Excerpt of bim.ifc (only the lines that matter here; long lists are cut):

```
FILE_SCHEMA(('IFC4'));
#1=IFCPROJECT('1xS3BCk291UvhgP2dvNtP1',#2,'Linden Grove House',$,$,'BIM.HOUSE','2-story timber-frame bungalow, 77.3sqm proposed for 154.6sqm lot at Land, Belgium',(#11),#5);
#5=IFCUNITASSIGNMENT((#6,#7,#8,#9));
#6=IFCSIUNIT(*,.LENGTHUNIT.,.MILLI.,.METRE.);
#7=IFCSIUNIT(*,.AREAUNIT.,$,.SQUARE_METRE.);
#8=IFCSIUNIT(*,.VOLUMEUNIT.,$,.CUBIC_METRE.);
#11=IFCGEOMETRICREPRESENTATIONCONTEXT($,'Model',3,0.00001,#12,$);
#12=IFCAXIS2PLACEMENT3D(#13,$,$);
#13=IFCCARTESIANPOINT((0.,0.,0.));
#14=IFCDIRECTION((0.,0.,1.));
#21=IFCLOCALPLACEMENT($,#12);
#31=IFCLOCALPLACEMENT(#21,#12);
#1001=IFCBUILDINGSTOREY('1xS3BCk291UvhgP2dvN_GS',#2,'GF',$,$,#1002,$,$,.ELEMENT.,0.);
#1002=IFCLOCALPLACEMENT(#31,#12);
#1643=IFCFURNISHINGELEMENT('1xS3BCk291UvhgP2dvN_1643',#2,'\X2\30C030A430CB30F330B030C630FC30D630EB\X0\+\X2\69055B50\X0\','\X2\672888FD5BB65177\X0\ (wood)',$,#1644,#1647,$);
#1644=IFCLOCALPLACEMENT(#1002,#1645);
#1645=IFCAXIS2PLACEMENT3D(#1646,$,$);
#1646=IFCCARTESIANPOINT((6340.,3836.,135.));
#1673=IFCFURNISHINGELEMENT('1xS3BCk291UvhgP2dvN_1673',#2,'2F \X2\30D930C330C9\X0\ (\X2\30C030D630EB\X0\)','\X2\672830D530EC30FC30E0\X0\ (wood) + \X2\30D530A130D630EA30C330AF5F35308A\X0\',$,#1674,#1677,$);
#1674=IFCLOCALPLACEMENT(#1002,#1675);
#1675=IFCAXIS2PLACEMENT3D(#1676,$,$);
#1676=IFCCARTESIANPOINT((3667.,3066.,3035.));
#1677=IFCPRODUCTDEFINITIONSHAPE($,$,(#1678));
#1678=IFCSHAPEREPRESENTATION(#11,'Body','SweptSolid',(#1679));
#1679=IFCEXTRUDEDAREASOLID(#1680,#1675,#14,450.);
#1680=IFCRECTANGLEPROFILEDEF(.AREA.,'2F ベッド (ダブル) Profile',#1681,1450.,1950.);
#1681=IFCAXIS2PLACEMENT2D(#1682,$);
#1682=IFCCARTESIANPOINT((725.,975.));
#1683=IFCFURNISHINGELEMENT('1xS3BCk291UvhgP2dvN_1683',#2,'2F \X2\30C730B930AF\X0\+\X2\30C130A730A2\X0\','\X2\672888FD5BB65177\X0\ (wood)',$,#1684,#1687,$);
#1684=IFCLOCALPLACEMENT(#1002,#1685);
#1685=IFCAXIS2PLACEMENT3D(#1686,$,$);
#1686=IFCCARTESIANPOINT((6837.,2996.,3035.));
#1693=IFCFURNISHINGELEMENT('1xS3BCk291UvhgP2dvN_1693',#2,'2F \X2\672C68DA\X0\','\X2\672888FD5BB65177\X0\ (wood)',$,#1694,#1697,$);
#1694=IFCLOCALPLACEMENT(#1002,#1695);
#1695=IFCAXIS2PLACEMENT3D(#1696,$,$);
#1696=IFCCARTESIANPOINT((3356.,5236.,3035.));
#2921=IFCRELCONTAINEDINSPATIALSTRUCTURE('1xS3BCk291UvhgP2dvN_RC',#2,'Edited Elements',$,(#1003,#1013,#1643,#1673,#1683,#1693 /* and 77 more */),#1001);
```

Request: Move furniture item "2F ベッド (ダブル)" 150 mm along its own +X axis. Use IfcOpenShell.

```python
import ifcopenshell
import ifcopenshell.api.geometry
import ifcopenshell.util.placement
import ifcopenshell.util.unit

model = ifcopenshell.open("bim.ifc")
unit_scale = ifcopenshell.util.unit.calculate_unit_scale(model)

item = model.by_id(1673)
matrix = ifcopenshell.util.placement.get_local_placement(item.ObjectPlacement)
matrix[:3, 3] += matrix[:3, 0] * 0.15 / unit_scale
ifcopenshell.api.geometry.edit_object_placement(model, product=item, matrix=matrix, is_si=False)

print(ifcopenshell.util.placement.get_local_placement(item.ObjectPlacement).round(3) + 0.0)

model.write("bim_edited.ifc")
```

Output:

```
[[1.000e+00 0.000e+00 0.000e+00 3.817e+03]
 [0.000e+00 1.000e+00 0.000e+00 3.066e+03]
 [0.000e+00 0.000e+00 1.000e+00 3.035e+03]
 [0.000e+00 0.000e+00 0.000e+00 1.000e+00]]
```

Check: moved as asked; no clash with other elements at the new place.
